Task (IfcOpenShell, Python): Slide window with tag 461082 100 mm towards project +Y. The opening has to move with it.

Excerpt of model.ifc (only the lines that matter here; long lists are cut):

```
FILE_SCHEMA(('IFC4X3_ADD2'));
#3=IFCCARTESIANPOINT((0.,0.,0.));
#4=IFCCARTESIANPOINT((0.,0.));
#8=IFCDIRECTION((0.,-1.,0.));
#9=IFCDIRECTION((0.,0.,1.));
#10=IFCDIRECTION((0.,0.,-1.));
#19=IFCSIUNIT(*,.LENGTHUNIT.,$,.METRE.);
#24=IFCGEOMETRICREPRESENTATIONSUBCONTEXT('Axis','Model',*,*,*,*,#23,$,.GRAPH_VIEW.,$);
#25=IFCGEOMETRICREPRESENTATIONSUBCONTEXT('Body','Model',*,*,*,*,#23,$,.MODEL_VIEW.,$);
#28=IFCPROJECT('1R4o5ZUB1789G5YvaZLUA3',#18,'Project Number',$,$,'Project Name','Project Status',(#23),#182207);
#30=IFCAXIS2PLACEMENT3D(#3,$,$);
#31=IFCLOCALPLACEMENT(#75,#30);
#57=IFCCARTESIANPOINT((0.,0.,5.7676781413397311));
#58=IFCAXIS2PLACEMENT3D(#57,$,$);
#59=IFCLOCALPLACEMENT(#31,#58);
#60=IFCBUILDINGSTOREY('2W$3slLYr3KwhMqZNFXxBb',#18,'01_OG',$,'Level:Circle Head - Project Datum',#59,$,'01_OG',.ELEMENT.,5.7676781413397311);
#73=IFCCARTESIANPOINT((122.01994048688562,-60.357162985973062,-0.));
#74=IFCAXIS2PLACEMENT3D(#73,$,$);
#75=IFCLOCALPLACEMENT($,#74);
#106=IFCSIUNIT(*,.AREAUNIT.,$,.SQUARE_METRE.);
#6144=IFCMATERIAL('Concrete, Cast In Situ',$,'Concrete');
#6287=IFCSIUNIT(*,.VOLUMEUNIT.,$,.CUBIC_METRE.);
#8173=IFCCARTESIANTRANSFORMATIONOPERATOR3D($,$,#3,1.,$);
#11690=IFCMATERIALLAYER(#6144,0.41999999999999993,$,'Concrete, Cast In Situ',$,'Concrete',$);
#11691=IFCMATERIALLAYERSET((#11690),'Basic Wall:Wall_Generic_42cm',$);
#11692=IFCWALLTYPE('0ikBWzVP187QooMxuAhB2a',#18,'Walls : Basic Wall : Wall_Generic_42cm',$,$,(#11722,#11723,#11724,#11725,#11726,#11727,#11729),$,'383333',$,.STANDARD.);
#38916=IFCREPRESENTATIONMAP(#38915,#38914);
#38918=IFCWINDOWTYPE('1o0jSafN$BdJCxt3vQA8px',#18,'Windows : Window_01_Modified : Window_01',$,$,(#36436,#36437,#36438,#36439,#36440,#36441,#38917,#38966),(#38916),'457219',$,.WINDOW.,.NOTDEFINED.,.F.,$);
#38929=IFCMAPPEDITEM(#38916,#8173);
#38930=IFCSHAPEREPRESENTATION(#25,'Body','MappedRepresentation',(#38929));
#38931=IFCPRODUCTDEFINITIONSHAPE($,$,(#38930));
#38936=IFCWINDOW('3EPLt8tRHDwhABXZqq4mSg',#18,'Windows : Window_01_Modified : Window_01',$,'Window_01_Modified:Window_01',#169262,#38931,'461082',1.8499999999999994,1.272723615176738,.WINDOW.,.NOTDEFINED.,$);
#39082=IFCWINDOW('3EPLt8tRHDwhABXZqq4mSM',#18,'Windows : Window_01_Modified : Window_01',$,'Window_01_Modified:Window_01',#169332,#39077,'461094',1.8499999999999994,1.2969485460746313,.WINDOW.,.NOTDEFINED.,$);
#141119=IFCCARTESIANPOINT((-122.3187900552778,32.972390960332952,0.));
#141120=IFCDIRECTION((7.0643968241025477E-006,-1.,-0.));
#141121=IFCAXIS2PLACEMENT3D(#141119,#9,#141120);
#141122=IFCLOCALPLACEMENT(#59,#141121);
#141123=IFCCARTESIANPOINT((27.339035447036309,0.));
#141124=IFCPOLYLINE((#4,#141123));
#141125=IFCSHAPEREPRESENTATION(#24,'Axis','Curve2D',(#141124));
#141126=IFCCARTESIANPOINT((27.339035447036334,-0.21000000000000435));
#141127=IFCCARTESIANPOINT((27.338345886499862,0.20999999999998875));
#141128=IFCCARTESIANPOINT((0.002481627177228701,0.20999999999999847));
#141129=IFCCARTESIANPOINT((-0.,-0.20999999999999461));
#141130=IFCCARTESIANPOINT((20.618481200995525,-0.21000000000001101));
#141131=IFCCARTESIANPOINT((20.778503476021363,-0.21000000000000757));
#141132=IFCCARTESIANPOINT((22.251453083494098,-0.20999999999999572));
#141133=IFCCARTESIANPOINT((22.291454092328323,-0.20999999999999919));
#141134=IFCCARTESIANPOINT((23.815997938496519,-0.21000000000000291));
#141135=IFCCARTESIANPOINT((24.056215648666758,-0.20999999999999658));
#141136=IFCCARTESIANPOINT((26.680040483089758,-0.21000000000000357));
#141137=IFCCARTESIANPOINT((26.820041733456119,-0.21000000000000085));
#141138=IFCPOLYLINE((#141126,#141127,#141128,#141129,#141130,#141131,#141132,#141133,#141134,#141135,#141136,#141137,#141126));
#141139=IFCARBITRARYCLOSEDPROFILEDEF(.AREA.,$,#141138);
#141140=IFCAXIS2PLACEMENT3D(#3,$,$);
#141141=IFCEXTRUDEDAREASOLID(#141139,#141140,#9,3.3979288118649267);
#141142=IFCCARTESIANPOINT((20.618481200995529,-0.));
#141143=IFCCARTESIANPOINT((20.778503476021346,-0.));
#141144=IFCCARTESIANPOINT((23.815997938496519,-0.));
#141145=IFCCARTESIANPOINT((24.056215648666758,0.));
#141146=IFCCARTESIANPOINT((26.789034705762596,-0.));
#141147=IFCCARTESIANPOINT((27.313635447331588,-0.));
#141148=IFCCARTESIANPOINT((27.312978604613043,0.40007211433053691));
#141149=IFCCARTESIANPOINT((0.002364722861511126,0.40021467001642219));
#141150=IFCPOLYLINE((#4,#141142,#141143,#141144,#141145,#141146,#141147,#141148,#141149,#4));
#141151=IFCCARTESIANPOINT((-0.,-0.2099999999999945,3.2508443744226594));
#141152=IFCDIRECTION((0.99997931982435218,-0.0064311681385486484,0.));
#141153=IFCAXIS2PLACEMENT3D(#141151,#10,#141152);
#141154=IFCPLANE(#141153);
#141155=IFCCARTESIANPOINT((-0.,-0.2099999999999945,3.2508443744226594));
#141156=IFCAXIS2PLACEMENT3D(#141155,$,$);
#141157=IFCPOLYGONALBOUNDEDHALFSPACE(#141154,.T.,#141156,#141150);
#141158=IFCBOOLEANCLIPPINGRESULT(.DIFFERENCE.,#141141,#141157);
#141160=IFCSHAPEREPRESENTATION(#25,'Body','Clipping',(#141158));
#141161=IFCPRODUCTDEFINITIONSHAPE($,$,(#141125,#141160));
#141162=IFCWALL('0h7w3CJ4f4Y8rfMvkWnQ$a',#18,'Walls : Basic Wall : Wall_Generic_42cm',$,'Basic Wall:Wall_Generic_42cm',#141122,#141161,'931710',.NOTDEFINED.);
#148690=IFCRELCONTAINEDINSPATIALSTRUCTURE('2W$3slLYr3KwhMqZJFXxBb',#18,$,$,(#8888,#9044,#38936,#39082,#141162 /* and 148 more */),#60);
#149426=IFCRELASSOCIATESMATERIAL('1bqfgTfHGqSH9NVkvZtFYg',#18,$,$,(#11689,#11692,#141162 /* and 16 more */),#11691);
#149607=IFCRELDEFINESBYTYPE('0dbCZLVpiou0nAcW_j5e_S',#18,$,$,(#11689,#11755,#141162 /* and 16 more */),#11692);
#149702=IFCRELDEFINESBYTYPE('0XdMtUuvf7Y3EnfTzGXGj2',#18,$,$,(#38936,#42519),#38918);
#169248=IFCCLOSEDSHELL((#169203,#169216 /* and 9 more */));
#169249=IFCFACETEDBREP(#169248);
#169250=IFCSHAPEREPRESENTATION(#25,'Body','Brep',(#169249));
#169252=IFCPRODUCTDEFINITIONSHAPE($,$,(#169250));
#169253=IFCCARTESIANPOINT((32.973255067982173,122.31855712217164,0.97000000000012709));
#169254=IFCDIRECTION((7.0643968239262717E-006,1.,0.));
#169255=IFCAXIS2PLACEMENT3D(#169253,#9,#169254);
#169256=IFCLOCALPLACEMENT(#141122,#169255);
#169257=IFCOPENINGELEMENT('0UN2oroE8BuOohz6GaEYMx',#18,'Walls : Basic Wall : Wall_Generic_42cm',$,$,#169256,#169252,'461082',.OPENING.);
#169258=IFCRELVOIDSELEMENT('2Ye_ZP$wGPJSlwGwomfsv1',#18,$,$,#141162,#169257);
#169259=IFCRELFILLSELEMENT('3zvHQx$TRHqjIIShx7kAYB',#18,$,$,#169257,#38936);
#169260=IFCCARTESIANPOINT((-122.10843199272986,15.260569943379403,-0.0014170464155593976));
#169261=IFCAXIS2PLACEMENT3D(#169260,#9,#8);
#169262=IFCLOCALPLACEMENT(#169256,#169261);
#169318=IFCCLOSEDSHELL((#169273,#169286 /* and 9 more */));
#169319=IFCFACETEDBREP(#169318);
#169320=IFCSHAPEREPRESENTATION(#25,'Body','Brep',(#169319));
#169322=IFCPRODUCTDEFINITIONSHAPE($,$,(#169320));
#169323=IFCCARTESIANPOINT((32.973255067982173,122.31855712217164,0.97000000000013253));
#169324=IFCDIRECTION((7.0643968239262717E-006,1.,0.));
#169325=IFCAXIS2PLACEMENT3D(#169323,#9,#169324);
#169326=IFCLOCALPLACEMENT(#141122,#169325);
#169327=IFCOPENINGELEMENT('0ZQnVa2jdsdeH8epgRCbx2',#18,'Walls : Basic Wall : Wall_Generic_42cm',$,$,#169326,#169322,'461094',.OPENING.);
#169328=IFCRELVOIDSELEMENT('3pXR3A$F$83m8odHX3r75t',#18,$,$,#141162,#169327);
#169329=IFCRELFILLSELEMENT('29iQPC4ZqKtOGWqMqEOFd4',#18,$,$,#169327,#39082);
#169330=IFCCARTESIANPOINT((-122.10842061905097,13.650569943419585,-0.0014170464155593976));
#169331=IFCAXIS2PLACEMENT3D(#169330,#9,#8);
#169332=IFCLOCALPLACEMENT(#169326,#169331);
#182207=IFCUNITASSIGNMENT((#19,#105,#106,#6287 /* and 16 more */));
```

```python
import ifcopenshell
import ifcopenshell.api.geometry
import ifcopenshell.util.placement
import ifcopenshell.util.unit

model = ifcopenshell.open("model.ifc")
unit_scale = ifcopenshell.util.unit.calculate_unit_scale(model)

window = model.by_id(38936)
opening = window.FillsVoids[0].RelatingOpeningElement
wall = opening.VoidsElements[0].RelatingBuildingElement

wall_matrix = ifcopenshell.util.placement.get_local_placement(wall.ObjectPlacement)
shift = wall_matrix[:3, 0] * -0.1 / unit_scale
before = ifcopenshell.util.placement.get_local_placement(window.ObjectPlacement)[:3, 3].copy()

# The window is placed relative to its opening, so it follows when the opening moves.
matrix = ifcopenshell.util.placement.get_local_placement(opening.ObjectPlacement)
matrix[:3, 3] += shift
ifcopenshell.api.geometry.edit_object_placement(
    model, product=opening, matrix=matrix, is_si=False, should_transform_children=True
)

after = ifcopenshell.util.placement.get_local_placement(window.ObjectPlacement)[:3, 3]
print("window moved by", (after - before).round(3) + 0.0)

model.write("model_rev.ifc")
```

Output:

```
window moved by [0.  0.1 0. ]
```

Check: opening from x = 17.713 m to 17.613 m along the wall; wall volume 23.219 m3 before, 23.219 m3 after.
